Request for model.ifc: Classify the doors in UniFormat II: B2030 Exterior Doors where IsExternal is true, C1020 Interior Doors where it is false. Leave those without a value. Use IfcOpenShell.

First a look at what the model holds.

```python
import ifcopenshell
import ifcopenshell.util.element

model = ifcopenshell.open("model.ifc")
print(model.schema)
print("classifications:", [c.Name for c in model.by_type("IfcClassification")])
values = [ifcopenshell.util.element.get_pset(e, "Pset_DoorCommon", "IsExternal") for e in model.by_type("IfcDoor")]
for value in (True, False, None):
    print("IsExternal", value, values.count(value))
```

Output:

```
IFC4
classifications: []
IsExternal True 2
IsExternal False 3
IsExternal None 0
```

```python
import ifcopenshell
import ifcopenshell.api.classification
import ifcopenshell.util.element

model = ifcopenshell.open("model.ifc")

system = ifcopenshell.api.classification.add_classification(model, classification="UniFormat II")

doors = model.by_type("IfcDoor")
external = {e: ifcopenshell.util.element.get_pset(e, "Pset_DoorCommon", "IsExternal") for e in doors}
for flag, code, name in ((True, "B2030", "Exterior Doors"), (False, "C1020", "Interior Doors")):
    products = [e for e in doors if external[e] is flag]
    ifcopenshell.api.classification.add_reference(
        model, products=products, classification=system, identification=code, name=name
    )
    print(code, len(products))

model.write("model_rev.ifc")
```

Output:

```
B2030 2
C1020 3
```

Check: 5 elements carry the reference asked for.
